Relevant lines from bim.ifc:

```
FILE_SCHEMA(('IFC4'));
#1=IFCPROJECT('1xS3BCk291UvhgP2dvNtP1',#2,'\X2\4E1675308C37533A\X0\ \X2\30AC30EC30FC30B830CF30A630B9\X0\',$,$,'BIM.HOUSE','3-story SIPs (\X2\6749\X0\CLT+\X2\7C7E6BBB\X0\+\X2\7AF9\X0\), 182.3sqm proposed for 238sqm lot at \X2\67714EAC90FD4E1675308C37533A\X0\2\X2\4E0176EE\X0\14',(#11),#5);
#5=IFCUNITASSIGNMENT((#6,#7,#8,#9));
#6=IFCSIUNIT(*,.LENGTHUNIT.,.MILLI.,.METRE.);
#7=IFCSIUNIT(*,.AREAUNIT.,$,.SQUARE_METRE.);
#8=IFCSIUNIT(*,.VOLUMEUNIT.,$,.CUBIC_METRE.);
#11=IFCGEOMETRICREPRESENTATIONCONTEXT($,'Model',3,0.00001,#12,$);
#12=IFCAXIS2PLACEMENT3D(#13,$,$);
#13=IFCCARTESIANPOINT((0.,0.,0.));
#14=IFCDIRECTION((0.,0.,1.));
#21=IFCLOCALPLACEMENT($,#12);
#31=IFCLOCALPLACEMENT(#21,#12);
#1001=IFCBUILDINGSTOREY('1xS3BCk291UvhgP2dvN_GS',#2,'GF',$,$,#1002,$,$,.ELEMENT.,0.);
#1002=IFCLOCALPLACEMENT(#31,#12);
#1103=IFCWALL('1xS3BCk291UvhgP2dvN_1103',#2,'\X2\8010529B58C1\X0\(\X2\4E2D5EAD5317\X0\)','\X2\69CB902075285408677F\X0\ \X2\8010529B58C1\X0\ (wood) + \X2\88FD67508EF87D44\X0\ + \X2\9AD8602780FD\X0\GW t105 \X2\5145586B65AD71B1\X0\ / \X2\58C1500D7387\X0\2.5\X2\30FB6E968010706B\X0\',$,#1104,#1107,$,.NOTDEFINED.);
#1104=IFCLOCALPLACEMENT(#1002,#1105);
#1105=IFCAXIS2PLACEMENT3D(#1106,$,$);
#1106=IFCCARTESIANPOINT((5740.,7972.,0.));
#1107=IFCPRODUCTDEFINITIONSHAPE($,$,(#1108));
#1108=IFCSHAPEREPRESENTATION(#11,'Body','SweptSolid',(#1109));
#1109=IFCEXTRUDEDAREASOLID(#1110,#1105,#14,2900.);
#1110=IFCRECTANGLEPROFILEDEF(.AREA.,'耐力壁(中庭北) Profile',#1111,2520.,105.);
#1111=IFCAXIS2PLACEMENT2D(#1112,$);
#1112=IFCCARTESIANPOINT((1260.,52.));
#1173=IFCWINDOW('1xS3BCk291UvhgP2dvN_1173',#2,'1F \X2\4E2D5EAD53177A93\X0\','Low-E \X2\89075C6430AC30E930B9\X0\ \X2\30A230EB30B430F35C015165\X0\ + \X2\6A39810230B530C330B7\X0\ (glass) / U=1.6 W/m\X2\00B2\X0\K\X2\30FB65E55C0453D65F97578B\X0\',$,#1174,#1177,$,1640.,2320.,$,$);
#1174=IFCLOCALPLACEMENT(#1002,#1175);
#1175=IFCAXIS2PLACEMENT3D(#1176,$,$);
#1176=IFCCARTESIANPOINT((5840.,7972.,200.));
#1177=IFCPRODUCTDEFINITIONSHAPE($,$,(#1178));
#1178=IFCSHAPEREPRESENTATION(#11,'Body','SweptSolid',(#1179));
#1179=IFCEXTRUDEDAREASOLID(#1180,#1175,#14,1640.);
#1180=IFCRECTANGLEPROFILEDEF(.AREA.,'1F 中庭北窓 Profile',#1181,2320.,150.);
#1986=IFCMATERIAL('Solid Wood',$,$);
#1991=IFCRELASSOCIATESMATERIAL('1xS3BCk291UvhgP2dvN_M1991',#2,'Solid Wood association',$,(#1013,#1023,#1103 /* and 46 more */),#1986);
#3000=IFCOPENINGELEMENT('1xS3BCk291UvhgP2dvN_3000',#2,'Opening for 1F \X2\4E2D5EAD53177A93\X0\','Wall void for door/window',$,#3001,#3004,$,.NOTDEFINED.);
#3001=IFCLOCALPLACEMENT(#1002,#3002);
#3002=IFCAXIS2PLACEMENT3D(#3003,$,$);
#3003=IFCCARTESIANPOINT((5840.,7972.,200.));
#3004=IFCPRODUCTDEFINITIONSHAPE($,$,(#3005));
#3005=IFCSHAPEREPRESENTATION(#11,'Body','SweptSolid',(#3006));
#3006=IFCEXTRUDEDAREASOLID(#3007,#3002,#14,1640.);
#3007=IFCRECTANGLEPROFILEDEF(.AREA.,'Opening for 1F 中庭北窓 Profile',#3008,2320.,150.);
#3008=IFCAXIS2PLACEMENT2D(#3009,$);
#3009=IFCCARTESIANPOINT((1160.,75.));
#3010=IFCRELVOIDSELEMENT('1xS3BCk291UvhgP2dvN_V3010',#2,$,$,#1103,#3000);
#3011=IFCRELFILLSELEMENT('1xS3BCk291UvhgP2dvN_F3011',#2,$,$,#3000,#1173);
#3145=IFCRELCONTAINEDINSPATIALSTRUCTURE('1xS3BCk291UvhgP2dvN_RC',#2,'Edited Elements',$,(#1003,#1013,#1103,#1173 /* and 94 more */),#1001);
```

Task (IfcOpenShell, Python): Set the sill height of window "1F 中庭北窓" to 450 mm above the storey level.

```python
import numpy as np
import ifcopenshell
import ifcopenshell.api.geometry
import ifcopenshell.geom
import ifcopenshell.util.element
import ifcopenshell.util.placement
import ifcopenshell.util.shape
import ifcopenshell.util.unit

model = ifcopenshell.open("bim.ifc")
unit_scale = ifcopenshell.util.unit.calculate_unit_scale(model)

window = model.by_guid("1xS3BCk291UvhgP2dvN_1173")
opening = window.FillsVoids[0].RelatingOpeningElement
storey = ifcopenshell.util.element.get_container(window, ifc_class="IfcBuildingStorey")
level = ifcopenshell.util.placement.get_local_placement(storey.ObjectPlacement)[2, 3]

# The opening's origin need not be at the sill, so measure its lowest point.
shape = ifcopenshell.geom.create_shape(ifcopenshell.geom.settings(), opening)
bottom = ifcopenshell.util.shape.get_shape_bottom_elevation(shape, shape.geometry) / unit_scale
dz = level + 0.45 / unit_scale - bottom

shift = np.array([0.0, 0.0, dz])
# The window is not placed relative to its opening, so move both.
for product in (opening, window):
    matrix = ifcopenshell.util.placement.get_local_placement(product.ObjectPlacement)
    matrix[:3, 3] += shift
    ifcopenshell.api.geometry.edit_object_placement(model, product=product, matrix=matrix, is_si=False)

print(f"moved by {dz * unit_scale:+.3f} m")

model.write("bim_updated.ifc")
```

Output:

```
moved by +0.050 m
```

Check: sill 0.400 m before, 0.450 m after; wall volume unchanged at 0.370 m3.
